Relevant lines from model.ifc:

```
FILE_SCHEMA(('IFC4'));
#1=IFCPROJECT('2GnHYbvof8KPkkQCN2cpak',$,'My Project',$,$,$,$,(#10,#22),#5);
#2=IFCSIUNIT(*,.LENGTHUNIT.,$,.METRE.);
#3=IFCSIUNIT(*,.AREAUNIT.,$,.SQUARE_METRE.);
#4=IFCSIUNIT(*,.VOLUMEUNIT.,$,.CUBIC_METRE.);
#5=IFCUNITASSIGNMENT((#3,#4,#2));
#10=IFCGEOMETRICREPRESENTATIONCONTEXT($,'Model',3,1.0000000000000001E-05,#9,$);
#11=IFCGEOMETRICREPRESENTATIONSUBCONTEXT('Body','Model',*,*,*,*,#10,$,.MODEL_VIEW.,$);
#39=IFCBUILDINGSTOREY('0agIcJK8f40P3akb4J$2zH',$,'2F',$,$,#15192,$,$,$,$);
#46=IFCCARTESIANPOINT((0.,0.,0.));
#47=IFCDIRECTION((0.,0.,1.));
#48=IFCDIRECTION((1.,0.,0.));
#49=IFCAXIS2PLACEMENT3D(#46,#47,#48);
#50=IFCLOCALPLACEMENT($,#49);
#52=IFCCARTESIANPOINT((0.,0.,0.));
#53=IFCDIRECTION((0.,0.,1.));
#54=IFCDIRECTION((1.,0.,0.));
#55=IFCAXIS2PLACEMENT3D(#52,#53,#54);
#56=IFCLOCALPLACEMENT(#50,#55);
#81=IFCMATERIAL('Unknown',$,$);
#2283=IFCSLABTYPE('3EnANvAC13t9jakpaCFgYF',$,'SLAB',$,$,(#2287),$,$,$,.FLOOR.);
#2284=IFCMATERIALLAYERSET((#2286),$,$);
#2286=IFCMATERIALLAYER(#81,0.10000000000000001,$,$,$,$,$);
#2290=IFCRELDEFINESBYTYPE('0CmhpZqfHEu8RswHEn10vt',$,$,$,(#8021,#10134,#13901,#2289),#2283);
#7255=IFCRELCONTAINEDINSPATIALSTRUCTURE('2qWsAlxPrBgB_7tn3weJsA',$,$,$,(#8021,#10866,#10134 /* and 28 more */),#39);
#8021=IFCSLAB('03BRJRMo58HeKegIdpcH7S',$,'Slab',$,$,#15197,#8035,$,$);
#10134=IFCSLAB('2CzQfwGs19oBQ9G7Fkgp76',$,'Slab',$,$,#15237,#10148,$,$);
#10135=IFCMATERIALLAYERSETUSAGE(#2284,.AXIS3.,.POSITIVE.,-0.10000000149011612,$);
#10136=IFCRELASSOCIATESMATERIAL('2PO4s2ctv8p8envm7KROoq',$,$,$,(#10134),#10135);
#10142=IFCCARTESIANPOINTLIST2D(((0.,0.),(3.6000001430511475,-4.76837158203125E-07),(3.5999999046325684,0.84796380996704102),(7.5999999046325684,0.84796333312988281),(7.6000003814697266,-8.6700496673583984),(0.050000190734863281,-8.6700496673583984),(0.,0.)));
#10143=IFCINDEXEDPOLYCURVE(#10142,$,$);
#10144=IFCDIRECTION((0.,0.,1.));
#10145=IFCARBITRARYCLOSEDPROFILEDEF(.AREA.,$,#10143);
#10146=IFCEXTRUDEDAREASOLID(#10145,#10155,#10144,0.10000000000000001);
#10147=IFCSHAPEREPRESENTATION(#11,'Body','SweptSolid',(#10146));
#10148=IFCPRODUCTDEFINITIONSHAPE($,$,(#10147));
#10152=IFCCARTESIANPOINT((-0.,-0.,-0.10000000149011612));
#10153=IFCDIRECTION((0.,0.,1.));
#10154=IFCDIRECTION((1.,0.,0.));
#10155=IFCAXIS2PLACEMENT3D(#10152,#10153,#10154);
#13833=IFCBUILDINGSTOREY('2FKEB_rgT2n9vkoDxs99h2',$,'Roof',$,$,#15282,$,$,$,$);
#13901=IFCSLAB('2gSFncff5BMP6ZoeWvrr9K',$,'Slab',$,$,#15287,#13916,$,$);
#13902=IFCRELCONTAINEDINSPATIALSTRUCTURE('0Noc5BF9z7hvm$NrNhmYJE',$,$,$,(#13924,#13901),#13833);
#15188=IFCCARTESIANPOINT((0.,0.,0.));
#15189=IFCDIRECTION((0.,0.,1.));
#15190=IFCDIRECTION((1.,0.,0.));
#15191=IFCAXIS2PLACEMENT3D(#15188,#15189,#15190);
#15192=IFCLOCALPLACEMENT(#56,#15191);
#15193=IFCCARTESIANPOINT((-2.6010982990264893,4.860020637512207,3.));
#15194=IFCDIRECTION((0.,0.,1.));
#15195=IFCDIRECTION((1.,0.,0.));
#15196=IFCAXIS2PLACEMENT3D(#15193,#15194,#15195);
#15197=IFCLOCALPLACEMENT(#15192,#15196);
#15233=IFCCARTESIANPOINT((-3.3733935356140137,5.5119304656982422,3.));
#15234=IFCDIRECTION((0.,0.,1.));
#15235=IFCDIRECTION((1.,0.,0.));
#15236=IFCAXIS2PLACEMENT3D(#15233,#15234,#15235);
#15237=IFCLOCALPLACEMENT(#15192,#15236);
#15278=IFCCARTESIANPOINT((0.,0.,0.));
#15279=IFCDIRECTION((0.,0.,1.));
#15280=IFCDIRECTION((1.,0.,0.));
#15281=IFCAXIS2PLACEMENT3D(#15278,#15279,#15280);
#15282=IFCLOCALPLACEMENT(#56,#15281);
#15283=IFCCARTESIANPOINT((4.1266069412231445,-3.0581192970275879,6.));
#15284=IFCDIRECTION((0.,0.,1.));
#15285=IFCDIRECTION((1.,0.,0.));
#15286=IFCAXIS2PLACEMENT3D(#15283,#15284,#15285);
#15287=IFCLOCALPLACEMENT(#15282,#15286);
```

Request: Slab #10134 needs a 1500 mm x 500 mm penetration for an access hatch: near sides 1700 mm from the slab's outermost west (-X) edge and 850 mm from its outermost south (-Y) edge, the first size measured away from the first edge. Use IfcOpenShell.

```python
import numpy as np
import ifcopenshell
import ifcopenshell.api.feature
import ifcopenshell.api.geometry
import ifcopenshell.api.root
import ifcopenshell.geom
import ifcopenshell.util.placement
import ifcopenshell.util.representation
import ifcopenshell.util.shape
import ifcopenshell.util.unit

model = ifcopenshell.open("model.ifc")
unit_scale = ifcopenshell.util.unit.calculate_unit_scale(model)
settings = ifcopenshell.geom.settings()


def volume(element):
    """Net volume in cubic metres, openings subtracted."""
    shape = ifcopenshell.geom.create_shape(settings, element)
    return ifcopenshell.util.shape.get_volume(shape.geometry)


slab = model.by_guid("2CzQfwGs19oBQ9G7Fkgp76")
before = volume(slab)

# Extent in the slab's own axes, in metres. The edges named are its -X and -Y sides.
slab_shape = ifcopenshell.geom.create_shape(settings, slab)
vertices = ifcopenshell.util.shape.get_vertices(slab_shape.geometry)
x_min, y_min, bottom = vertices.min(axis=0)
top = vertices[:, 2].max()

opening = ifcopenshell.api.root.create_entity(model, ifc_class="IfcOpeningElement", name="Access hatch opening", predefined_type="OPENING")
context = ifcopenshell.util.representation.get_context(model, "Model", "Body", "MODEL_VIEW")
width, depth = 1.5, 0.5
outline = [(0.0, 0.0), (width, 0.0), (width, depth), (0.0, depth), (0.0, 0.0)]
# Overshoot both faces by 50 mm so the cut is clean.
shape = ifcopenshell.api.geometry.add_slab_representation(
    model, context=context, depth=top - bottom + 0.1, polyline=outline
)
ifcopenshell.api.geometry.assign_representation(model, product=opening, representation=shape)

matrix = ifcopenshell.util.placement.get_local_placement(slab.ObjectPlacement)
matrix[:, 3] = matrix @ np.append(np.array([x_min + 1.7, y_min + 0.85, bottom - 0.05]) / unit_scale, 1.0)
ifcopenshell.api.geometry.edit_object_placement(model, product=opening, matrix=matrix, is_si=False)
ifcopenshell.api.feature.add_feature(model, feature=opening, element=slab)

after = volume(slab)

print(f"slab volume {before:.3f} -> {after:.3f} m3")

model.write("model_rev.ifc")
```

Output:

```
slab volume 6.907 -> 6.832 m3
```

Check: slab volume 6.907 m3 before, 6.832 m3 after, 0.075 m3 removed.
